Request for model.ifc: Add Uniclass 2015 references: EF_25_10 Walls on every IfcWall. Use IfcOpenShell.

First a look at what the model holds.

```python
import ifcopenshell

model = ifcopenshell.open("model.ifc")
print(model.schema)
print("classifications:", [c.Name for c in model.by_type("IfcClassification")])
for ifc_class in ("IfcDoor", "IfcRoof", "IfcStair", "IfcWall", "IfcWindow"):
    print(ifc_class, len(model.by_type(ifc_class)))
```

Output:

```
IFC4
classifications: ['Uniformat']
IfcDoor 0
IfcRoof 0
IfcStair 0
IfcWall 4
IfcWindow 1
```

```python
import ifcopenshell
import ifcopenshell.api.classification

model = ifcopenshell.open("model.ifc")

system = ifcopenshell.api.classification.add_classification(model, classification="Uniclass 2015")

codes = {
    "IfcWall": ("EF_25_10", "Walls"),
}
for ifc_class, (code, name) in codes.items():
    products = model.by_type(ifc_class)
    ifcopenshell.api.classification.add_reference(
        model, products=products, classification=system, identification=code, name=name
    )
    print(code, len(products))

model.write("model_rev.ifc")
```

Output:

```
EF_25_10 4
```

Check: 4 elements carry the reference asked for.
